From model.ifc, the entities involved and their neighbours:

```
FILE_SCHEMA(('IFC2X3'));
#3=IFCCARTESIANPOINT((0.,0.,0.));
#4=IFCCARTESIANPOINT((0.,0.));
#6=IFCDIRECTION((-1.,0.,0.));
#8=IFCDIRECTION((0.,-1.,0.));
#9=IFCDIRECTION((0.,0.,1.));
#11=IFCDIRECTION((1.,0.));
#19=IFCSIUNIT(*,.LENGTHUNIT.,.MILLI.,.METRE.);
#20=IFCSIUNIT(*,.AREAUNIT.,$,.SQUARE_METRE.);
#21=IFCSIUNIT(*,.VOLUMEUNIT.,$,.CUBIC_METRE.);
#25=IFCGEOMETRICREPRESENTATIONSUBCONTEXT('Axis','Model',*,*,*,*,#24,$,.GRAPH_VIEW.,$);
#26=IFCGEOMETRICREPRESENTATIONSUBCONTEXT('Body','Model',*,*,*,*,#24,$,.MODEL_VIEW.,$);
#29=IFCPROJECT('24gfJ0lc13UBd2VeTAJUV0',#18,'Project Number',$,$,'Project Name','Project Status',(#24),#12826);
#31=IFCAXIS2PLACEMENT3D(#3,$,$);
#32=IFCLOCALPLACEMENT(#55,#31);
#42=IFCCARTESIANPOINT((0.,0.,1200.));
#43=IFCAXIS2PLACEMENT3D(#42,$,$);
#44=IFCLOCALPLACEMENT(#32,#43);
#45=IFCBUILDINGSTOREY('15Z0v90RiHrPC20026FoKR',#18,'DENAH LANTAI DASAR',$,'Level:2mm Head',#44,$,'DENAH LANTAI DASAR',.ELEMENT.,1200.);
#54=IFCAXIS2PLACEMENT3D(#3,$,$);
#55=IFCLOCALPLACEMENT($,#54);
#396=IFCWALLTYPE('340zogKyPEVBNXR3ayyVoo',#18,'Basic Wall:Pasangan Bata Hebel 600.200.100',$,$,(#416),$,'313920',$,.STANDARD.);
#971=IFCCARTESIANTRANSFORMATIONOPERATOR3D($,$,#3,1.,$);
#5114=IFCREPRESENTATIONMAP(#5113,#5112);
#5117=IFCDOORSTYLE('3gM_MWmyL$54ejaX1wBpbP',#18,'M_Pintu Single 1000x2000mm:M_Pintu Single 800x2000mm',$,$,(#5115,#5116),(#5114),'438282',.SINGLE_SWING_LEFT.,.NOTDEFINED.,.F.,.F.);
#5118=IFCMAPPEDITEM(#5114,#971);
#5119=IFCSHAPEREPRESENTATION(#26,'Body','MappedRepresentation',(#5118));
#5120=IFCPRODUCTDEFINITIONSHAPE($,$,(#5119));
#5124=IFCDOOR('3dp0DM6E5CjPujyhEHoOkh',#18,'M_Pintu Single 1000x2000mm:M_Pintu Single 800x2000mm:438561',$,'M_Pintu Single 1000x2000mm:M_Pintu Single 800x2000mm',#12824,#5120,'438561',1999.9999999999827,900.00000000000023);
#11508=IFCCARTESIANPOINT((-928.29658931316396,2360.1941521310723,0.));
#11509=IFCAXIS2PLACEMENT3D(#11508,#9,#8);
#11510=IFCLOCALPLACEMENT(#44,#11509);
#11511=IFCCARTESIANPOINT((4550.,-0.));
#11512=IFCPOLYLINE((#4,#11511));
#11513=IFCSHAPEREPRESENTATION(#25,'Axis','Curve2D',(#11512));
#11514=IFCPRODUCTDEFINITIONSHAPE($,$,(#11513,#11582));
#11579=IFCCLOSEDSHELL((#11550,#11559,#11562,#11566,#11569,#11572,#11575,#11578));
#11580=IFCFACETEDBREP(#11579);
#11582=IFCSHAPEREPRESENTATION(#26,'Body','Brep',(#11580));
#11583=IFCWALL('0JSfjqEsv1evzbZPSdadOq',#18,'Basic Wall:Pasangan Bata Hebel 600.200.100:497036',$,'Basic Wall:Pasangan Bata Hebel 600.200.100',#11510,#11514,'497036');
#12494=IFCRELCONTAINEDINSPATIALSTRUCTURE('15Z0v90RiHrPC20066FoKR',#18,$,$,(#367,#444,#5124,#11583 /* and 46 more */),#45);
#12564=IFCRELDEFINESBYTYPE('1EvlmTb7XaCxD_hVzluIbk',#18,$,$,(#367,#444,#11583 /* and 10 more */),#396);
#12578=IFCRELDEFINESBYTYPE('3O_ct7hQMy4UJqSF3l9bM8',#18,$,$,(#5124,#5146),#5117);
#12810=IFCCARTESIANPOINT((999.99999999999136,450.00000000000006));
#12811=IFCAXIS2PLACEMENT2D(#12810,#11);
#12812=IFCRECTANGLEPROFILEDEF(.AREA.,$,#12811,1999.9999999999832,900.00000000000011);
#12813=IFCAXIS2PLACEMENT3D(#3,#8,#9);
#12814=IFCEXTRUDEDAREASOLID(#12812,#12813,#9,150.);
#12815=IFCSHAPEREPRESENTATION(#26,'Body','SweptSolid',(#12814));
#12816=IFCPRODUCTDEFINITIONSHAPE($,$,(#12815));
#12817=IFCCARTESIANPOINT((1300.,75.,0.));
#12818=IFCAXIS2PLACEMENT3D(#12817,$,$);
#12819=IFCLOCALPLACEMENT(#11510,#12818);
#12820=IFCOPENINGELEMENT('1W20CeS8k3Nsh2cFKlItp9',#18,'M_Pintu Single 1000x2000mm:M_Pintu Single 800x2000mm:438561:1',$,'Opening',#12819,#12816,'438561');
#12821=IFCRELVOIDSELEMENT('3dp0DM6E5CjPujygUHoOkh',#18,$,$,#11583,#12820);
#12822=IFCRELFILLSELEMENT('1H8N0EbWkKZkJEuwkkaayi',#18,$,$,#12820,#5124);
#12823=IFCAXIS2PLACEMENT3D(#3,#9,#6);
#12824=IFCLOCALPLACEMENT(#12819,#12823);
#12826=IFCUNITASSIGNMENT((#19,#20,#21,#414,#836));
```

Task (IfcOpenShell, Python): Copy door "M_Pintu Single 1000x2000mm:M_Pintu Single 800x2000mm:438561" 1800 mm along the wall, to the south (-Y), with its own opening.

```python
import ifcopenshell
import ifcopenshell.api.feature
import ifcopenshell.api.geometry
import ifcopenshell.api.root
import ifcopenshell.geom
import ifcopenshell.util.element
import ifcopenshell.util.placement
import ifcopenshell.util.shape
import ifcopenshell.util.unit

model = ifcopenshell.open("model.ifc")
unit_scale = ifcopenshell.util.unit.calculate_unit_scale(model)
settings = ifcopenshell.geom.settings()


def volume(element):
    """Net volume in cubic metres, openings subtracted."""
    shape = ifcopenshell.geom.create_shape(settings, element)
    return ifcopenshell.util.shape.get_volume(shape.geometry)


def reuse_history(source, copy):
    """copy_class also copies each property set's owner history, people and application; keep the originals."""
    for rel in copy.IsDefinedBy:
        if rel.is_a("IfcRelDefinesByProperties") and (history := rel.RelatingPropertyDefinition.OwnerHistory):
            rel.RelatingPropertyDefinition.OwnerHistory = source.OwnerHistory
            ifcopenshell.util.element.remove_deep2(model, history)


door = model.by_guid("3dp0DM6E5CjPujyhEHoOkh")
opening = door.FillsVoids[0].RelatingOpeningElement
wall = opening.VoidsElements[0].RelatingBuildingElement
before = volume(wall)
shift = ifcopenshell.util.placement.get_local_placement(wall.ObjectPlacement)[:3, 0] * 1.8 / unit_scale

# copy_class copies the void relationship, type, container and properties, but no geometry.
new_opening = ifcopenshell.api.root.copy_class(model, product=opening)
new_opening.Representation = ifcopenshell.util.element.copy_deep(
    model, opening.Representation, exclude=["IfcGeometricRepresentationContext", "IfcRepresentationMap"]
)
new_opening.Name = "M_Pintu Single 1000x2000mm:M_Pintu Single 800x2000mm"
new_opening.Tag = None
new_door = ifcopenshell.api.root.copy_class(model, product=door)
new_door.Representation = ifcopenshell.util.element.copy_deep(
    model, door.Representation, exclude=["IfcGeometricRepresentationContext", "IfcRepresentationMap"]
)
new_door.Name = "M_Pintu Single 1000x2000mm:M_Pintu Single 800x2000mm"
new_door.Tag = None
reuse_history(door, new_door)
fills = ifcopenshell.api.feature.add_filling(model, opening=new_opening, element=new_door)
fills.OwnerHistory = new_door.OwnerHistory  # required in IFC2X3

for old, new in ((opening, new_opening), (door, new_door)):
    matrix = ifcopenshell.util.placement.get_local_placement(old.ObjectPlacement)
    matrix[:3, 3] += shift
    ifcopenshell.api.geometry.edit_object_placement(model, product=new, matrix=matrix, is_si=False)

after = volume(wall)

print(f"wall volume {before:.3f} -> {after:.3f} m3")

model.write("model_v2.ifc")
```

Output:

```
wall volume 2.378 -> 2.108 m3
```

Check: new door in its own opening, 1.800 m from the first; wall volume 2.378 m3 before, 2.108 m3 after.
